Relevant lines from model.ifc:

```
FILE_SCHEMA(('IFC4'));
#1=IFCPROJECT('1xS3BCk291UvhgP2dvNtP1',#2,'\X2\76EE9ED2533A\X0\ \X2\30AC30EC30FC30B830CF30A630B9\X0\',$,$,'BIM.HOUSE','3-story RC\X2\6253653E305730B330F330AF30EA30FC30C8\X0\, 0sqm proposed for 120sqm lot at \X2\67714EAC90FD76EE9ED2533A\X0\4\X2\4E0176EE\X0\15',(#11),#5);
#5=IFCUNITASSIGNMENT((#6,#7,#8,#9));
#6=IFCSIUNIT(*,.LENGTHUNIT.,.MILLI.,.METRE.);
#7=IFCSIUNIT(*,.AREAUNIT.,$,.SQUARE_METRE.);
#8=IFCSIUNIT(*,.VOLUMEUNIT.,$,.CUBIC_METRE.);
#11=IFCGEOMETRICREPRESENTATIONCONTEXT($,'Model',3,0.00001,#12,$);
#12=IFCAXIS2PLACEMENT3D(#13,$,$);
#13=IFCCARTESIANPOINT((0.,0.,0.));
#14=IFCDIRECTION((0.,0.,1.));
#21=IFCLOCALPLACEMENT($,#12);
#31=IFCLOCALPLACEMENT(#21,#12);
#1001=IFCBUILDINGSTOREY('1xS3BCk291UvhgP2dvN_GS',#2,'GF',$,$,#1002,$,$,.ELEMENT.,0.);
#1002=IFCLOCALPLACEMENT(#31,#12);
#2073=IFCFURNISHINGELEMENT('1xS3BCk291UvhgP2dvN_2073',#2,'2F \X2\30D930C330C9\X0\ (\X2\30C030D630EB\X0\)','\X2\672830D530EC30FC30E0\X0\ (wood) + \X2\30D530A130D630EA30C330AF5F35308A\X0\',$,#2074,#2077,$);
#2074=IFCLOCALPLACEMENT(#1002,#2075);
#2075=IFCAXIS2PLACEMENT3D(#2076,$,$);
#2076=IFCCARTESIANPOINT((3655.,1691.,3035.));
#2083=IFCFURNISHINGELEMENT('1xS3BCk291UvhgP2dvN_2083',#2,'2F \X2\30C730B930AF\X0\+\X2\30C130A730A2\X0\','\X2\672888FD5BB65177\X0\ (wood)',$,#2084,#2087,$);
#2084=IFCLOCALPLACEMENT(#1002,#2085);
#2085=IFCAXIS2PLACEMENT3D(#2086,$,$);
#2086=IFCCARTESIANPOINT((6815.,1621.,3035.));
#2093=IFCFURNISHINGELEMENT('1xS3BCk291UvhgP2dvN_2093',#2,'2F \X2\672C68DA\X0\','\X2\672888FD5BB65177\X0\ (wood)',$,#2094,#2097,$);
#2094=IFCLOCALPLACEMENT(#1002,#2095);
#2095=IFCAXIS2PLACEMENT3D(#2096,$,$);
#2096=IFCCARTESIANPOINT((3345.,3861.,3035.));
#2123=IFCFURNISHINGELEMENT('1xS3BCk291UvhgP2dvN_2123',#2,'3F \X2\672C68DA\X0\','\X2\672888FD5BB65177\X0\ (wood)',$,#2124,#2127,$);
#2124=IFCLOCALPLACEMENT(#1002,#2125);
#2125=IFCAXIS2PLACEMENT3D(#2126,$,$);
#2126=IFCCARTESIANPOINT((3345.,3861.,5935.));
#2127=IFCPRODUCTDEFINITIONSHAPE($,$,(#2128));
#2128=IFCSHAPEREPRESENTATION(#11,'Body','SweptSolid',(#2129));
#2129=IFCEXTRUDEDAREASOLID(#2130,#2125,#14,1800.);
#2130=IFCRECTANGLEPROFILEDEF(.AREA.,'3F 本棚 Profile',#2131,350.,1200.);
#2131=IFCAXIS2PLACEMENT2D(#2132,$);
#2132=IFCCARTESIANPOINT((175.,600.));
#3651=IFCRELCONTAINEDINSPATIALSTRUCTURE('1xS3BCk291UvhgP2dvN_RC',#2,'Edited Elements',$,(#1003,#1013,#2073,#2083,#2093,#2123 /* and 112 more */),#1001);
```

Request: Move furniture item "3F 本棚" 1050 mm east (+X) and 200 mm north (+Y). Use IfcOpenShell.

```python
import ifcopenshell
import ifcopenshell.api.geometry
import ifcopenshell.util.placement
import ifcopenshell.util.unit

model = ifcopenshell.open("model.ifc")
unit_scale = ifcopenshell.util.unit.calculate_unit_scale(model)

item = model.by_guid("1xS3BCk291UvhgP2dvN_2123")
matrix = ifcopenshell.util.placement.get_local_placement(item.ObjectPlacement)
matrix[0, 3] += 1.05 / unit_scale
matrix[1, 3] += 0.2 / unit_scale
ifcopenshell.api.geometry.edit_object_placement(model, product=item, matrix=matrix, is_si=False)

print(ifcopenshell.util.placement.get_local_placement(item.ObjectPlacement).round(3) + 0.0)

model.write("model_updated.ifc")
```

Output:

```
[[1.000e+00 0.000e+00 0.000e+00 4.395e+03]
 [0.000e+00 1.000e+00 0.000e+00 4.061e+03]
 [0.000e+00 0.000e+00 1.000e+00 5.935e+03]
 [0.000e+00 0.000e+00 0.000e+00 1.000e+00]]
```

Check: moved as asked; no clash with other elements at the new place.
